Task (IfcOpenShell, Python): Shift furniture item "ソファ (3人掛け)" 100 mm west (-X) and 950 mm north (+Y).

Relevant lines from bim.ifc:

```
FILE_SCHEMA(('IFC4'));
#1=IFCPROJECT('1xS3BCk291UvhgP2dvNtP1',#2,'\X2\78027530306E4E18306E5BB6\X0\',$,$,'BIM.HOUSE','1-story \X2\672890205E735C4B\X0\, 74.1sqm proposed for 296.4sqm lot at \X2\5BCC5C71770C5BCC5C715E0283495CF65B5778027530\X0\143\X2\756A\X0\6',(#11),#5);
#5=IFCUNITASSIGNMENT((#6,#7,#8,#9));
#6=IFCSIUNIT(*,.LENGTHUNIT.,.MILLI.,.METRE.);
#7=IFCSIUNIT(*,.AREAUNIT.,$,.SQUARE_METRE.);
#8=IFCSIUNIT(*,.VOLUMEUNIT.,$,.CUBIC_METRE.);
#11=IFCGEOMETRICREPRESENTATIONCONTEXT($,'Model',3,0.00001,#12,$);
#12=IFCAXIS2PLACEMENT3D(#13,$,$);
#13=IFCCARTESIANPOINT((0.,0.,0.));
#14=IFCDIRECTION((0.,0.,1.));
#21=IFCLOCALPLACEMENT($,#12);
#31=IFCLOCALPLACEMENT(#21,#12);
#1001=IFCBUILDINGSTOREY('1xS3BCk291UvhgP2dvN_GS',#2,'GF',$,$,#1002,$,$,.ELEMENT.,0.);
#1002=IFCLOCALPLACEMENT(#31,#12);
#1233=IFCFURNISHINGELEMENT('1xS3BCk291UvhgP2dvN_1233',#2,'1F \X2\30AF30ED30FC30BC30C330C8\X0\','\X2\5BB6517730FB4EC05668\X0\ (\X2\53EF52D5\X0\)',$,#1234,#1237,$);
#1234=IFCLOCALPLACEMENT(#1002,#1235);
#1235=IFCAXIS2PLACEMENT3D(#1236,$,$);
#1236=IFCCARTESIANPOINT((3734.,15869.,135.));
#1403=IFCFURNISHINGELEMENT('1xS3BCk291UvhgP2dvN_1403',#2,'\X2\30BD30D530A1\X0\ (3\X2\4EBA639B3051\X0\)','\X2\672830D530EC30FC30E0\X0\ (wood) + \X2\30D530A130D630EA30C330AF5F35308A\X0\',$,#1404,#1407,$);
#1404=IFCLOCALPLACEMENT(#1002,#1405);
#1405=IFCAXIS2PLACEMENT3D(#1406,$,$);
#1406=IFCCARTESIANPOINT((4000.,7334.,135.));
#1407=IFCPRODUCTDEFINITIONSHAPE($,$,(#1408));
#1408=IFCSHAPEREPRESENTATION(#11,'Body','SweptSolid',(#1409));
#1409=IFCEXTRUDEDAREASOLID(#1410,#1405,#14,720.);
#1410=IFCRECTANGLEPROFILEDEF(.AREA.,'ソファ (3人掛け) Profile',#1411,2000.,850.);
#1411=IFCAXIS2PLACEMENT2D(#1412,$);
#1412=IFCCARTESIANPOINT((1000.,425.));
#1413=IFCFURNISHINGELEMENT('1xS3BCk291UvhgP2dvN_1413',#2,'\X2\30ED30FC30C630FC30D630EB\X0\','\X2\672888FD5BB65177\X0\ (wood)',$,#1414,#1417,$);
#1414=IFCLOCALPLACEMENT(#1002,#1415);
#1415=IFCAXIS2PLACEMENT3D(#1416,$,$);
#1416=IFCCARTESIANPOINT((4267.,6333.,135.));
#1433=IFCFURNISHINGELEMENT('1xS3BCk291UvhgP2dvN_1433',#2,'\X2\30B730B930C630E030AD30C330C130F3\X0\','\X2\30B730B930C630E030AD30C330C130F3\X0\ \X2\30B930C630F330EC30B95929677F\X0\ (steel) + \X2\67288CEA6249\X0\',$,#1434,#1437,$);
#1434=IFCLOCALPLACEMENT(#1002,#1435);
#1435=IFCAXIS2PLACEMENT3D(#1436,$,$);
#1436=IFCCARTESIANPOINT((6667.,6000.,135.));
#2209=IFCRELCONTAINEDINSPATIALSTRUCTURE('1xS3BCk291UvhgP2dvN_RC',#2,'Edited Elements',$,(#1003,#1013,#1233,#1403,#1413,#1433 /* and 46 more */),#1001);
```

```python
import ifcopenshell
import ifcopenshell.api.geometry
import ifcopenshell.util.placement

model = ifcopenshell.open("bim.ifc")

item = model.by_guid("1xS3BCk291UvhgP2dvN_1403")
matrix = ifcopenshell.util.placement.get_local_placement(item.ObjectPlacement)
matrix[0, 3] -= 100.0
matrix[1, 3] += 950.0
ifcopenshell.api.geometry.edit_object_placement(model, product=item, matrix=matrix, is_si=False)

print(ifcopenshell.util.placement.get_local_placement(item.ObjectPlacement).round(3) + 0.0)

model.write("bim_rev.ifc")
```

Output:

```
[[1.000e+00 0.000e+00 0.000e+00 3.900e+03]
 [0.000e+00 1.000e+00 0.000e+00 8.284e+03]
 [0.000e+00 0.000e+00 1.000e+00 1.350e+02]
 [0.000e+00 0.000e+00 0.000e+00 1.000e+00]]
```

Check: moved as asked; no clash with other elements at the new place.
